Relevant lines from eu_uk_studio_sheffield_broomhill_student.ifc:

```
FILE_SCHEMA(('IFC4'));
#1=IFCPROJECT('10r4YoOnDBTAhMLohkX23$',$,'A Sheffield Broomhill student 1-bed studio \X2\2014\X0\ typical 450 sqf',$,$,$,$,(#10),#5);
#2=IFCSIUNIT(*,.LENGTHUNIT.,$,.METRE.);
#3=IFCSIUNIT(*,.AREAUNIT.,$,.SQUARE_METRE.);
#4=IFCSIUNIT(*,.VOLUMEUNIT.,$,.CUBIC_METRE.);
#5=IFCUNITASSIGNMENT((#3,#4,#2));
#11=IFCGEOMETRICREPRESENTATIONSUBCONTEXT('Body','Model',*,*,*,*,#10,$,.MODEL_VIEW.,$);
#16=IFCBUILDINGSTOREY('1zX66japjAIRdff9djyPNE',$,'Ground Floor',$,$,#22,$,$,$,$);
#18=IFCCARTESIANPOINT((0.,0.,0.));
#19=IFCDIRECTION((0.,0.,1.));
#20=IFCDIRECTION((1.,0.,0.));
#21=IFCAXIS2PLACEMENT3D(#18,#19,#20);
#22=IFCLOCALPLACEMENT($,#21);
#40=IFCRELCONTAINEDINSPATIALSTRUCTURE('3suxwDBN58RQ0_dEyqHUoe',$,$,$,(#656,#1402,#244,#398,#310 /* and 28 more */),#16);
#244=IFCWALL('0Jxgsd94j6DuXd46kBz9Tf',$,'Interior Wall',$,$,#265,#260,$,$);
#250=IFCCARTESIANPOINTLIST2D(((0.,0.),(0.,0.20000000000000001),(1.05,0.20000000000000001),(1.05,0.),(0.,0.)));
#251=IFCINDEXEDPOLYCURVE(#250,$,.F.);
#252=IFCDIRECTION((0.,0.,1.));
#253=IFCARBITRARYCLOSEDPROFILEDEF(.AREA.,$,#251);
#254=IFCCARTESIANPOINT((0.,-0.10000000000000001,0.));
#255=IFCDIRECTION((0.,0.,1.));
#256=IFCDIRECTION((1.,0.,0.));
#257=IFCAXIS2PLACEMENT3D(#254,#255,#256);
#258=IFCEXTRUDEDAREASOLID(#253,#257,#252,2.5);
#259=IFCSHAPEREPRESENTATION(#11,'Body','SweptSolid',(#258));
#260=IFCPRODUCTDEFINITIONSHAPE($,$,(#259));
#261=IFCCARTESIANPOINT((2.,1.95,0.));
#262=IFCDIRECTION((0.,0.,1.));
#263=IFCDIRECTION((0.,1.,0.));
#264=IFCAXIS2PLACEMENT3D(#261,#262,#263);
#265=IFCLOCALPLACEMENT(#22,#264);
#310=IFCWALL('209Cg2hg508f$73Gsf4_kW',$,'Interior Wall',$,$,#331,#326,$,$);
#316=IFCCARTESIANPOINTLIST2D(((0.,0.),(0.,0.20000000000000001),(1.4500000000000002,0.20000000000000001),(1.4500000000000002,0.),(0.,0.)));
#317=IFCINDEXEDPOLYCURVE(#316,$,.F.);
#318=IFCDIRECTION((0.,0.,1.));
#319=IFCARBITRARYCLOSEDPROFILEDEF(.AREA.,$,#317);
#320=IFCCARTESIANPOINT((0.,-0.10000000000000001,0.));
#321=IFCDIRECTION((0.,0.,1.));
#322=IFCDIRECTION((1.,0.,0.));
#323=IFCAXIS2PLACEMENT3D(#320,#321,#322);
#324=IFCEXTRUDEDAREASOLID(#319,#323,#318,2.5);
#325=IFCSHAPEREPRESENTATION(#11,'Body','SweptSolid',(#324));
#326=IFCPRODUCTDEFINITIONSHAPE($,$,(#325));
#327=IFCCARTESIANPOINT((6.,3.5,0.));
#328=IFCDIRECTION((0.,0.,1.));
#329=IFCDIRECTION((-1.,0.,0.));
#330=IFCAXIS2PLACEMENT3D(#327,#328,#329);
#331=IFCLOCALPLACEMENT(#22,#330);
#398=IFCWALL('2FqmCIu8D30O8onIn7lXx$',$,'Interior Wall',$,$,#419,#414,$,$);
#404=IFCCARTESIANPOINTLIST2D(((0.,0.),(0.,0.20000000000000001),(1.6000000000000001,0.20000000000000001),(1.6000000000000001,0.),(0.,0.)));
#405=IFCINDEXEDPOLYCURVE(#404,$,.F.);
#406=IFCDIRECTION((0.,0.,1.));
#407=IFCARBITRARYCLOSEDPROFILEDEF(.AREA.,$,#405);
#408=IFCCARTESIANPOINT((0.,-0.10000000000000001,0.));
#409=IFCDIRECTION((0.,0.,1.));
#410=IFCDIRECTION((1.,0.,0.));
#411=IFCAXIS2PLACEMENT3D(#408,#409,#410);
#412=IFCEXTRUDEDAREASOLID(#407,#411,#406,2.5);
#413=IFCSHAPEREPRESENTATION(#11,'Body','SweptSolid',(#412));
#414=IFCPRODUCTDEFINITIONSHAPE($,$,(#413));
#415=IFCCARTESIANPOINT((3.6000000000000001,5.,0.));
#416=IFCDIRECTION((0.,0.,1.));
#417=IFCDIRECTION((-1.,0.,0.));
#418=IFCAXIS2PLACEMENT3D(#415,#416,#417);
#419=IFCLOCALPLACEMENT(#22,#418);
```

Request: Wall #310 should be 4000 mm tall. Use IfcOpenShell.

```python
import ifcopenshell
import ifcopenshell.geom
import ifcopenshell.util.representation
import ifcopenshell.util.shape

model = ifcopenshell.open("eu_uk_studio_sheffield_broomhill_student.ifc")
settings = ifcopenshell.geom.settings()


def volume(element):
    """Net volume in cubic metres, openings subtracted."""
    shape = ifcopenshell.geom.create_shape(settings, element)
    return ifcopenshell.util.shape.get_volume(shape.geometry)


wall = model.by_guid("209Cg2hg508f$73Gsf4_kW")
before = volume(wall)

body = ifcopenshell.util.representation.get_representation(wall, "Model", "Body")
solid = body.Items[0]
old_height = solid.Depth
solid.Depth = 4.0
after = volume(wall)

print(f"height {old_height:g} -> {solid.Depth:g}, volume {before:.3f} -> {after:.3f} m3")

model.write("eu_uk_studio_sheffield_broomhill_student_rev.ifc")
```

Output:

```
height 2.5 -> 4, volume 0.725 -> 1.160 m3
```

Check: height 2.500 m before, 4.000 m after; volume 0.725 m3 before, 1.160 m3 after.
